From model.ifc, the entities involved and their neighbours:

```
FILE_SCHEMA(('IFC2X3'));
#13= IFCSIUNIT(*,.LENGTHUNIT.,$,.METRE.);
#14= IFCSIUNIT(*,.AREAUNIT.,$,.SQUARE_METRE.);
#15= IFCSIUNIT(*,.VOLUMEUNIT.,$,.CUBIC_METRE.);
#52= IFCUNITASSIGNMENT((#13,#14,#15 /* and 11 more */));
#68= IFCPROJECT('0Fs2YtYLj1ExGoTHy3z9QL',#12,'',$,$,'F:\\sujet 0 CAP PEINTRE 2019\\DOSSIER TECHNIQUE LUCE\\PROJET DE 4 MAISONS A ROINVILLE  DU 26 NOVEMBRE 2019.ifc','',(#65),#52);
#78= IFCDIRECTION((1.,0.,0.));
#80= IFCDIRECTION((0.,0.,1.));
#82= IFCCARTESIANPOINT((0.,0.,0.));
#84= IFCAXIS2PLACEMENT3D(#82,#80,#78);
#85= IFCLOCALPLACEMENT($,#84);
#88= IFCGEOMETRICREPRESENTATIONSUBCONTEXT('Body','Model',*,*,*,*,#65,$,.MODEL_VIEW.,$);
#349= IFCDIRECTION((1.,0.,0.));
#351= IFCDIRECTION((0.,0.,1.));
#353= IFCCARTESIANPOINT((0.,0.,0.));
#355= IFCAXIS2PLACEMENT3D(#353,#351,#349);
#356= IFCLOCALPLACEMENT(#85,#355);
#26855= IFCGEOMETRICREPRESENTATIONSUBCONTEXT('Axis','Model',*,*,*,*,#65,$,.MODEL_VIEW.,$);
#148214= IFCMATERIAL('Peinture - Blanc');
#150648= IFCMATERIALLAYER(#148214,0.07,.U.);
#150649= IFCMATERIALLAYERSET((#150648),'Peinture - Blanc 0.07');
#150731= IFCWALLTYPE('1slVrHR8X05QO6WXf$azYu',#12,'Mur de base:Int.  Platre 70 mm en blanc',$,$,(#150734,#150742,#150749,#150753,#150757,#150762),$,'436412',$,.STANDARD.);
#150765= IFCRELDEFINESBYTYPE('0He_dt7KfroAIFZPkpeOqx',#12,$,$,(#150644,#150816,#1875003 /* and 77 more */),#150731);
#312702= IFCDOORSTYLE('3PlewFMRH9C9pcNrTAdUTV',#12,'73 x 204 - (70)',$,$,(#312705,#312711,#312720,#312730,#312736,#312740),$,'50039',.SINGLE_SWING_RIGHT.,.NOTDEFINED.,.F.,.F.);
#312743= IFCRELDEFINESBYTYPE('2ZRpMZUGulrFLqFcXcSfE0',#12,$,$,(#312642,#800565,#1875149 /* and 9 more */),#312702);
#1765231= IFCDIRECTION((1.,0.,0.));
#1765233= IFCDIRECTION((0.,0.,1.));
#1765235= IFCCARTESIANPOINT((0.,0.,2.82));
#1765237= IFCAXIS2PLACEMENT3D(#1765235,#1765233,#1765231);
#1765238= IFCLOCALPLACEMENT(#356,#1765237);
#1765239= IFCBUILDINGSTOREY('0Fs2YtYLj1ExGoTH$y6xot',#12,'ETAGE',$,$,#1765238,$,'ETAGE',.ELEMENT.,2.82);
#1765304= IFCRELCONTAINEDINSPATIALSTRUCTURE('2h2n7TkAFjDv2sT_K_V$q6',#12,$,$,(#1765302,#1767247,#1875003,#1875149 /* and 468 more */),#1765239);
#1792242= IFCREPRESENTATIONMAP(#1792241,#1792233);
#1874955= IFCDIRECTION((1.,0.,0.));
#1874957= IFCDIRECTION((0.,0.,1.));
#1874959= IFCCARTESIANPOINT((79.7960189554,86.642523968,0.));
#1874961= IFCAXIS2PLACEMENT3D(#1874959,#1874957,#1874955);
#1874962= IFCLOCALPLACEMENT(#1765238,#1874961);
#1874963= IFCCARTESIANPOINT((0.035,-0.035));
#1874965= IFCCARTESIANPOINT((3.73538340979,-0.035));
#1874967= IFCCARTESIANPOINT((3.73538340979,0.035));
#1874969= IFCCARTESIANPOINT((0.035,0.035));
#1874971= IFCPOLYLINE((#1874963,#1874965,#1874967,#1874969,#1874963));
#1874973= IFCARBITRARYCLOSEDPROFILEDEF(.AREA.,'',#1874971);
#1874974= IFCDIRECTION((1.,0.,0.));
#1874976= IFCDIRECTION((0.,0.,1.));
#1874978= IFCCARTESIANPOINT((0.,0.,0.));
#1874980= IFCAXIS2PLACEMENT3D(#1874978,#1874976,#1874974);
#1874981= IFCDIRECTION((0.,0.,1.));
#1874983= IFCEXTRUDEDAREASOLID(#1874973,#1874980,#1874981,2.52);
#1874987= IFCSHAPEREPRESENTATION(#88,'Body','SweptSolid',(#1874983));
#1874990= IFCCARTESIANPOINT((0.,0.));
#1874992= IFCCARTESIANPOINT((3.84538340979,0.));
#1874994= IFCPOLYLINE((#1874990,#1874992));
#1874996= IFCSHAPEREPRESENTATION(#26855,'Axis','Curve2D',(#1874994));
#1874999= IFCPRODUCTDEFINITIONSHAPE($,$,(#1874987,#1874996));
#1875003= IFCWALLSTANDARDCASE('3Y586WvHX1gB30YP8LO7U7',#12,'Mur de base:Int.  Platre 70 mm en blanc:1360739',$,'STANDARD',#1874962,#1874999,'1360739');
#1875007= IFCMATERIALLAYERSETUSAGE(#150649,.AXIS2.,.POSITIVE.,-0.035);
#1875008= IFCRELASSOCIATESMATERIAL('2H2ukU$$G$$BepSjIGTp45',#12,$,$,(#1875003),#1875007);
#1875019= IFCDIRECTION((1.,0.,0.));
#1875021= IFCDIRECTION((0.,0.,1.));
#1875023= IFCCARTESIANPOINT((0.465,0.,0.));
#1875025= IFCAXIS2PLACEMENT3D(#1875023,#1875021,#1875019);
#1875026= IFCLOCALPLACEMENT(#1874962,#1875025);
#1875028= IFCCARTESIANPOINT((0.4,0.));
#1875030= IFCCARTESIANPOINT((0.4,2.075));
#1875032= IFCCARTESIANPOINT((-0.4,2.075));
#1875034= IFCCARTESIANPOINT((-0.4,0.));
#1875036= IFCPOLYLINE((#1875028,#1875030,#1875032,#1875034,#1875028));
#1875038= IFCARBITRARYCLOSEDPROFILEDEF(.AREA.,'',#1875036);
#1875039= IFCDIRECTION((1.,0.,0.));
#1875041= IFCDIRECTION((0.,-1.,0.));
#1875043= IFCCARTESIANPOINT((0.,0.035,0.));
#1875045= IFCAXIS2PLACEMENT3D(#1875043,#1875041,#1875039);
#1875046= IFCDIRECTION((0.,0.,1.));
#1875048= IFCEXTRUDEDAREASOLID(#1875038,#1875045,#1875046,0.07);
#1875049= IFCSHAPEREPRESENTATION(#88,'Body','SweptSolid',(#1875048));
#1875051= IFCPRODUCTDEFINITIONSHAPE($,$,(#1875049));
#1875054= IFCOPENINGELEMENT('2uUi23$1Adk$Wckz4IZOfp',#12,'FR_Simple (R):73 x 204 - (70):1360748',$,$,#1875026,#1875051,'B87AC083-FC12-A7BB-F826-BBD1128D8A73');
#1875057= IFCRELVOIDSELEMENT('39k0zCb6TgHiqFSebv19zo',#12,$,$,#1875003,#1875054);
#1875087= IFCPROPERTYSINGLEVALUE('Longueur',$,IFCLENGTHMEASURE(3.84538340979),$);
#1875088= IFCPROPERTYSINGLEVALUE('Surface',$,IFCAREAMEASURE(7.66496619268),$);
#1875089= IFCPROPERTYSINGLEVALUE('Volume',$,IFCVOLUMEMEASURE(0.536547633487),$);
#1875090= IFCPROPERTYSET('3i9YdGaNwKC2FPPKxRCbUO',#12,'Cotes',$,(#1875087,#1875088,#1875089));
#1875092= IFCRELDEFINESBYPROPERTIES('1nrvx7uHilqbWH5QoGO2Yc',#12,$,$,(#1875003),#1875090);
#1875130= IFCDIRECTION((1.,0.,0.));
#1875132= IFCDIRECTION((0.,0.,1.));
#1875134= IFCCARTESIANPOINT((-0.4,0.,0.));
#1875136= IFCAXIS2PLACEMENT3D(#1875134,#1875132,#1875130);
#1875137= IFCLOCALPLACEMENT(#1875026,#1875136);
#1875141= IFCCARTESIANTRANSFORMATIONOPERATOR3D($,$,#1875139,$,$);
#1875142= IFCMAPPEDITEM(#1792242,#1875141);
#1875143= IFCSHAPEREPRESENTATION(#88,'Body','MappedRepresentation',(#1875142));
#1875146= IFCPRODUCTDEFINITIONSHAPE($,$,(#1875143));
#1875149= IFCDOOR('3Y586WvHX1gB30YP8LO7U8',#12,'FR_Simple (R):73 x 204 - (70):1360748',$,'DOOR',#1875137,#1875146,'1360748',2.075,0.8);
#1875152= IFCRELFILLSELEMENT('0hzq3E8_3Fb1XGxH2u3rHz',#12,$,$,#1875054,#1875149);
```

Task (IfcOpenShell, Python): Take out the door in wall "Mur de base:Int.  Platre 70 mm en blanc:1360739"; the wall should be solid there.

```python
import ifcopenshell
import ifcopenshell.api.feature
import ifcopenshell.api.pset
import ifcopenshell.api.root
import ifcopenshell.geom
import ifcopenshell.util.element
import ifcopenshell.util.shape
import ifcopenshell.util.unit

model = ifcopenshell.open("model.ifc")
area_scale = ifcopenshell.util.unit.calculate_unit_scale(model, "AREAUNIT")
volume_scale = ifcopenshell.util.unit.calculate_unit_scale(model, "VOLUMEUNIT")
settings = ifcopenshell.geom.settings()


def volume(element):
    """Net volume in cubic metres, openings subtracted."""
    shape = ifcopenshell.geom.create_shape(settings, element)
    return ifcopenshell.util.shape.get_volume(shape.geometry)


door = model.by_id(1875149)
opening = door.FillsVoids[0].RelatingOpeningElement
wall = opening.VoidsElements[0].RelatingBuildingElement
before = volume(wall)

ifcopenshell.api.root.remove_product(model, product=door)
ifcopenshell.api.feature.remove_feature(model, feature=opening)

after = volume(wall)
thickness = 0.07  # wall thickness in metres

# Update the wall's stored quantities.
pset = model.by_id(ifcopenshell.util.element.get_pset(wall, "Cotes", should_inherit=False)["id"])
ifcopenshell.api.pset.edit_pset(model, pset=pset, properties={
    "Surface": model.create_entity("IfcAreaMeasure", after / thickness / area_scale),
    "Volume": model.create_entity("IfcVolumeMeasure", after / volume_scale),
})

print(f"wall volume {before:.3f} -> {after:.3f} m3")

model.write("model_v2.ifc")
```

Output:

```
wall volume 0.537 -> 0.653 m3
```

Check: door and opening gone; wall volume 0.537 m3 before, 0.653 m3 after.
